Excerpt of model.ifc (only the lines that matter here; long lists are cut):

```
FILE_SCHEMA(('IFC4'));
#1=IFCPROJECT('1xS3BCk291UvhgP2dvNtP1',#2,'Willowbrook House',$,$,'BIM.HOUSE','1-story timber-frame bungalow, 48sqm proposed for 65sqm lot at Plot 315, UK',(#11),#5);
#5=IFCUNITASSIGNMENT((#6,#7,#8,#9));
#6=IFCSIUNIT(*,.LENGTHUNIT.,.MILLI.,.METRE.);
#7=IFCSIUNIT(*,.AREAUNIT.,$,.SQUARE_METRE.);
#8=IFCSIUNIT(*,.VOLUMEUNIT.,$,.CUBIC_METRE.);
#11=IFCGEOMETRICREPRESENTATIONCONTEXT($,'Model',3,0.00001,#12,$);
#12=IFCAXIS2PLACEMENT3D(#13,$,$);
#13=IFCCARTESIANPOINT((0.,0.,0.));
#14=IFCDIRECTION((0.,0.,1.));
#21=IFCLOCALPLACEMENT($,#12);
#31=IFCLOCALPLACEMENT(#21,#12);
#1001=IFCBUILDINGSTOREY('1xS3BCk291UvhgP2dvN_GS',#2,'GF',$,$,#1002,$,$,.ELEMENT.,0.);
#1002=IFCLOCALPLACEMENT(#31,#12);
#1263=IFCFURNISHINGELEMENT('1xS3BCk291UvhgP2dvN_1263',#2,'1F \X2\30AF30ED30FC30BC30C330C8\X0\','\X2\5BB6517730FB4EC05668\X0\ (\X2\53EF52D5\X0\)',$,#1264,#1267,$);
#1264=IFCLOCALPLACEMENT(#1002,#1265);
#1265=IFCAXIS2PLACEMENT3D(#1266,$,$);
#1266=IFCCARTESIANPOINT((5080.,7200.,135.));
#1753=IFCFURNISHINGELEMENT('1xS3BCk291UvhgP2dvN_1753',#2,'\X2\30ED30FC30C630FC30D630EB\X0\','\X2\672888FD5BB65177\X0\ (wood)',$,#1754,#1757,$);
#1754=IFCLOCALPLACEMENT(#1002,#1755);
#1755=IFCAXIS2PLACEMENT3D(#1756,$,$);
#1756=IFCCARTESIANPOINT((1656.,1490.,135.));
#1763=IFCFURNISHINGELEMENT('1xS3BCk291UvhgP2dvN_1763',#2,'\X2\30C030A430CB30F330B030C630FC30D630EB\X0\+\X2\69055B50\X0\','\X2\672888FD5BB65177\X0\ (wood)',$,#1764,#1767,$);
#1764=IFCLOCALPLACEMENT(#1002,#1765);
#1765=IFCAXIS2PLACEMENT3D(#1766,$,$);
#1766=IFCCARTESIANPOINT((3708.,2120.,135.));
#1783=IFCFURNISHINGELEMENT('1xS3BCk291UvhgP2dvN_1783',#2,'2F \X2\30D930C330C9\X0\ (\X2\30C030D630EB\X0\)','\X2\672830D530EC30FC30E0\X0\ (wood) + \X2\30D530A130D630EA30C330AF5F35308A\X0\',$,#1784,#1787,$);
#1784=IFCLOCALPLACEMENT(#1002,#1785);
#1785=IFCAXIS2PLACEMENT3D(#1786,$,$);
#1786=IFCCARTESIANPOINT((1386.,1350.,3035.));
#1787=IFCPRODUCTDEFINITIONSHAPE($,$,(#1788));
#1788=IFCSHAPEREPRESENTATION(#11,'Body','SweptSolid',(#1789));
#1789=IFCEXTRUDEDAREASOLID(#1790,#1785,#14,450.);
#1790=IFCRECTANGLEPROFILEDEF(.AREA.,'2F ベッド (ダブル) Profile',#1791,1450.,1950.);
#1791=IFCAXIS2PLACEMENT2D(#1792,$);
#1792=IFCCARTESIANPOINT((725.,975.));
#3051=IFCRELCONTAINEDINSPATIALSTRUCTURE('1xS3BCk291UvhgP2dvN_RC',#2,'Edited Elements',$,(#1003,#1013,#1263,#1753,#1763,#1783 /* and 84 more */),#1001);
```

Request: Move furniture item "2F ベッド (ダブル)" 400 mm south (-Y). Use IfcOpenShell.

```python
import ifcopenshell
import ifcopenshell.api.geometry
import ifcopenshell.util.placement
import ifcopenshell.util.unit

model = ifcopenshell.open("model.ifc")
unit_scale = ifcopenshell.util.unit.calculate_unit_scale(model)

item = model.by_guid("1xS3BCk291UvhgP2dvN_1783")
matrix = ifcopenshell.util.placement.get_local_placement(item.ObjectPlacement)
matrix[1, 3] -= 0.4 / unit_scale
ifcopenshell.api.geometry.edit_object_placement(model, product=item, matrix=matrix, is_si=False)

print(ifcopenshell.util.placement.get_local_placement(item.ObjectPlacement).round(3) + 0.0)

model.write("model-out.ifc")
```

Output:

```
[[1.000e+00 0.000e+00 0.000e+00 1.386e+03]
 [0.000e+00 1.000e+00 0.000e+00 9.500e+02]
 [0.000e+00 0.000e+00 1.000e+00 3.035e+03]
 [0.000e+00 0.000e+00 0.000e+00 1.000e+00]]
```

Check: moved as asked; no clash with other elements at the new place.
